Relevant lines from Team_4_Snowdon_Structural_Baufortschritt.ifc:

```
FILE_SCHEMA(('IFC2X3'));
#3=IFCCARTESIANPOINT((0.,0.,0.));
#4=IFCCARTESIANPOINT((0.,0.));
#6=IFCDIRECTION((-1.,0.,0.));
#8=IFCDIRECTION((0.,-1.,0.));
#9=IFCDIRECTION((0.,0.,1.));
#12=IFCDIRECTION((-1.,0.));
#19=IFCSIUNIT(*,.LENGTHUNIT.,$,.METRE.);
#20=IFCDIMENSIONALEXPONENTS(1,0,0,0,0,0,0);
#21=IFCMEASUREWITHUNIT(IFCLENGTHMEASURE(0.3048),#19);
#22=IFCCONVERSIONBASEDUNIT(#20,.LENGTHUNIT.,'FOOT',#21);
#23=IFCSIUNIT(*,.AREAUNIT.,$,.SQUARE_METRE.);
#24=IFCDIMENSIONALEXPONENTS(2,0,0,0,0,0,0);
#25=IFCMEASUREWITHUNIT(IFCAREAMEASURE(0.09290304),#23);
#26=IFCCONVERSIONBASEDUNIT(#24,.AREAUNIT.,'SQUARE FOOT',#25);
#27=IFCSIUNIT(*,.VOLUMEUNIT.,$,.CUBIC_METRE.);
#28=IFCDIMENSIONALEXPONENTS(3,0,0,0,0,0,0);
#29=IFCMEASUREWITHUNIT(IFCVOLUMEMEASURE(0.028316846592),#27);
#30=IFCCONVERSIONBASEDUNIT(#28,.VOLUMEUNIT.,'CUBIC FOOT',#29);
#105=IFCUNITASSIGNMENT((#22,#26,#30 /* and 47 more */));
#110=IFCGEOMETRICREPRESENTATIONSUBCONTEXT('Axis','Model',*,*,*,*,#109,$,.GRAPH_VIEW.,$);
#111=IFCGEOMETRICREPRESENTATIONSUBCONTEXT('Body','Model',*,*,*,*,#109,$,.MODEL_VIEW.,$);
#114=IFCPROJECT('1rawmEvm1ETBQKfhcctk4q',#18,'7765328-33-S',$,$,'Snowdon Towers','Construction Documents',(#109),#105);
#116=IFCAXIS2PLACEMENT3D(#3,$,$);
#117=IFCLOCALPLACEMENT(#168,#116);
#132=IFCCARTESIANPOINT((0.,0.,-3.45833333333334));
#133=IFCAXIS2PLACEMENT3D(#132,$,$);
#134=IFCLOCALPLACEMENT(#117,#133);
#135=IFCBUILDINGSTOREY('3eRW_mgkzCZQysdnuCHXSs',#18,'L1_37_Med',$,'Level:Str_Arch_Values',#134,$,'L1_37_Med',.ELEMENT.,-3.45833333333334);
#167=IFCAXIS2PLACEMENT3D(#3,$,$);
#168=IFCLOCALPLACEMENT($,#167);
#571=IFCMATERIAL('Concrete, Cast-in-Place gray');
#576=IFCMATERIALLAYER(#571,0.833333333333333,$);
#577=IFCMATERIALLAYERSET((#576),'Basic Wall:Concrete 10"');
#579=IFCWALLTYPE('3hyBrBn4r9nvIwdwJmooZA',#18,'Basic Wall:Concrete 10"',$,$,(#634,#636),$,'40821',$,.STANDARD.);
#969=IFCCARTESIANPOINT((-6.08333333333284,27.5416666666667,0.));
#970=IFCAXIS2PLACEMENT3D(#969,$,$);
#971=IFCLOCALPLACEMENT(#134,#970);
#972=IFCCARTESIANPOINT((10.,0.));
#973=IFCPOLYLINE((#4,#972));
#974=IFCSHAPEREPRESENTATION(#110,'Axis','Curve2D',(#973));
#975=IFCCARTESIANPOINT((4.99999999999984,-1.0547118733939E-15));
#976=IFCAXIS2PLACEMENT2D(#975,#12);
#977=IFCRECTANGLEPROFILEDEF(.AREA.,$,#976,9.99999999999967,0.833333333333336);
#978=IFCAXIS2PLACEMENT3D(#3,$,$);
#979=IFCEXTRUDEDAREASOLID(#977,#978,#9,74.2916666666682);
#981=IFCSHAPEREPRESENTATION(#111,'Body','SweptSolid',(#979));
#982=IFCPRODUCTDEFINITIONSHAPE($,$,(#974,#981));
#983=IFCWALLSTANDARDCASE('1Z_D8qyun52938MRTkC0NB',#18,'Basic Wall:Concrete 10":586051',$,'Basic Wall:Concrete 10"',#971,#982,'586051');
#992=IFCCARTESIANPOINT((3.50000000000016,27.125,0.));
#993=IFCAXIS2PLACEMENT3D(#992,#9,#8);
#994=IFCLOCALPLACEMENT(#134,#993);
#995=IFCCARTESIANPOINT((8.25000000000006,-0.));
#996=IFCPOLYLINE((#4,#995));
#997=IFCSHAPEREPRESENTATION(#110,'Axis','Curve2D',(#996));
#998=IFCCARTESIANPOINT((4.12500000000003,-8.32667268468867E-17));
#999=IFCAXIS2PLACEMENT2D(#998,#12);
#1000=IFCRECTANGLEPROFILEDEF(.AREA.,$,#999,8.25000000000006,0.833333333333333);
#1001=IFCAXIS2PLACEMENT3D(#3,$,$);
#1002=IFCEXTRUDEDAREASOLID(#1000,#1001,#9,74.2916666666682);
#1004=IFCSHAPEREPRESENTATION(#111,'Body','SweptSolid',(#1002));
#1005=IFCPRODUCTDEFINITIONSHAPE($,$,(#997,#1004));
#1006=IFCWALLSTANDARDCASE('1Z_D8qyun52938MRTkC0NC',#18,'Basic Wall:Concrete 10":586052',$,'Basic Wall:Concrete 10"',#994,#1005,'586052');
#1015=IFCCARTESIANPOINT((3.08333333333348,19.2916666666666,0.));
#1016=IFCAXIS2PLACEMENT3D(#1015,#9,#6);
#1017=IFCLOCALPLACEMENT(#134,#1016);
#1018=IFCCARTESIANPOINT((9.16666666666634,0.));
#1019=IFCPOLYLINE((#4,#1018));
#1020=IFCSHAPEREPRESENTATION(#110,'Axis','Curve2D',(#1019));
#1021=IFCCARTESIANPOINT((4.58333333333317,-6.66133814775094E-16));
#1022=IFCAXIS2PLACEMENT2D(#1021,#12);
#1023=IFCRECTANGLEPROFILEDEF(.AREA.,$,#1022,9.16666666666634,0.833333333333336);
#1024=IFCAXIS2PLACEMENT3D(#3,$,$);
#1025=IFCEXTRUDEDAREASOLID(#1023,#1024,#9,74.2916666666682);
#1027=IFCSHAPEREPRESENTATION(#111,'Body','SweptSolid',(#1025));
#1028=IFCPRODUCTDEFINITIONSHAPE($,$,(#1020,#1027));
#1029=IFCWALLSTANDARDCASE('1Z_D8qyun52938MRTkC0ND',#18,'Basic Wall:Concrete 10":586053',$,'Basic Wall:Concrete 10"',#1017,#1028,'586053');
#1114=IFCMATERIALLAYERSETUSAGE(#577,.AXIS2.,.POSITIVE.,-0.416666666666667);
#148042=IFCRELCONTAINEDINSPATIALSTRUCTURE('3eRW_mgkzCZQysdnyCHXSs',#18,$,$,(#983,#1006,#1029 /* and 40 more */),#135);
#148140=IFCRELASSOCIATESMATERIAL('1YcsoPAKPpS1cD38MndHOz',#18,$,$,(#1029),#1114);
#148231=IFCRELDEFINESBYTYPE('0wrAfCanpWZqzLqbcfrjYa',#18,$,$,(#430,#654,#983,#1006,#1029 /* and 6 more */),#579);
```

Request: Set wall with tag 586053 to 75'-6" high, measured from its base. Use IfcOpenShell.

```python
import ifcopenshell
import ifcopenshell.geom
import ifcopenshell.util.representation
import ifcopenshell.util.shape
import ifcopenshell.util.unit

model = ifcopenshell.open("Team_4_Snowdon_Structural_Baufortschritt.ifc")
unit_scale = ifcopenshell.util.unit.calculate_unit_scale(model)
settings = ifcopenshell.geom.settings()


def volume(element):
    """Net volume in cubic metres, openings subtracted."""
    shape = ifcopenshell.geom.create_shape(settings, element)
    return ifcopenshell.util.shape.get_volume(shape.geometry)


wall = model.by_guid("1Z_D8qyun52938MRTkC0ND")
before = volume(wall)

body = ifcopenshell.util.representation.get_representation(wall, "Model", "Body")
solid = body.Items[0]
old_height = solid.Depth
solid.Depth = 906 * 0.0254 / unit_scale
after = volume(wall)

print(f"height {old_height:g} -> {solid.Depth:g}, volume {before:.3f} -> {after:.3f} m3")

model.write("Team_4_Snowdon_Structural_Baufortschritt_v2.ifc")
```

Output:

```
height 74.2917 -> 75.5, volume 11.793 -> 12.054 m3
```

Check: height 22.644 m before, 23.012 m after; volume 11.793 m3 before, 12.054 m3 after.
